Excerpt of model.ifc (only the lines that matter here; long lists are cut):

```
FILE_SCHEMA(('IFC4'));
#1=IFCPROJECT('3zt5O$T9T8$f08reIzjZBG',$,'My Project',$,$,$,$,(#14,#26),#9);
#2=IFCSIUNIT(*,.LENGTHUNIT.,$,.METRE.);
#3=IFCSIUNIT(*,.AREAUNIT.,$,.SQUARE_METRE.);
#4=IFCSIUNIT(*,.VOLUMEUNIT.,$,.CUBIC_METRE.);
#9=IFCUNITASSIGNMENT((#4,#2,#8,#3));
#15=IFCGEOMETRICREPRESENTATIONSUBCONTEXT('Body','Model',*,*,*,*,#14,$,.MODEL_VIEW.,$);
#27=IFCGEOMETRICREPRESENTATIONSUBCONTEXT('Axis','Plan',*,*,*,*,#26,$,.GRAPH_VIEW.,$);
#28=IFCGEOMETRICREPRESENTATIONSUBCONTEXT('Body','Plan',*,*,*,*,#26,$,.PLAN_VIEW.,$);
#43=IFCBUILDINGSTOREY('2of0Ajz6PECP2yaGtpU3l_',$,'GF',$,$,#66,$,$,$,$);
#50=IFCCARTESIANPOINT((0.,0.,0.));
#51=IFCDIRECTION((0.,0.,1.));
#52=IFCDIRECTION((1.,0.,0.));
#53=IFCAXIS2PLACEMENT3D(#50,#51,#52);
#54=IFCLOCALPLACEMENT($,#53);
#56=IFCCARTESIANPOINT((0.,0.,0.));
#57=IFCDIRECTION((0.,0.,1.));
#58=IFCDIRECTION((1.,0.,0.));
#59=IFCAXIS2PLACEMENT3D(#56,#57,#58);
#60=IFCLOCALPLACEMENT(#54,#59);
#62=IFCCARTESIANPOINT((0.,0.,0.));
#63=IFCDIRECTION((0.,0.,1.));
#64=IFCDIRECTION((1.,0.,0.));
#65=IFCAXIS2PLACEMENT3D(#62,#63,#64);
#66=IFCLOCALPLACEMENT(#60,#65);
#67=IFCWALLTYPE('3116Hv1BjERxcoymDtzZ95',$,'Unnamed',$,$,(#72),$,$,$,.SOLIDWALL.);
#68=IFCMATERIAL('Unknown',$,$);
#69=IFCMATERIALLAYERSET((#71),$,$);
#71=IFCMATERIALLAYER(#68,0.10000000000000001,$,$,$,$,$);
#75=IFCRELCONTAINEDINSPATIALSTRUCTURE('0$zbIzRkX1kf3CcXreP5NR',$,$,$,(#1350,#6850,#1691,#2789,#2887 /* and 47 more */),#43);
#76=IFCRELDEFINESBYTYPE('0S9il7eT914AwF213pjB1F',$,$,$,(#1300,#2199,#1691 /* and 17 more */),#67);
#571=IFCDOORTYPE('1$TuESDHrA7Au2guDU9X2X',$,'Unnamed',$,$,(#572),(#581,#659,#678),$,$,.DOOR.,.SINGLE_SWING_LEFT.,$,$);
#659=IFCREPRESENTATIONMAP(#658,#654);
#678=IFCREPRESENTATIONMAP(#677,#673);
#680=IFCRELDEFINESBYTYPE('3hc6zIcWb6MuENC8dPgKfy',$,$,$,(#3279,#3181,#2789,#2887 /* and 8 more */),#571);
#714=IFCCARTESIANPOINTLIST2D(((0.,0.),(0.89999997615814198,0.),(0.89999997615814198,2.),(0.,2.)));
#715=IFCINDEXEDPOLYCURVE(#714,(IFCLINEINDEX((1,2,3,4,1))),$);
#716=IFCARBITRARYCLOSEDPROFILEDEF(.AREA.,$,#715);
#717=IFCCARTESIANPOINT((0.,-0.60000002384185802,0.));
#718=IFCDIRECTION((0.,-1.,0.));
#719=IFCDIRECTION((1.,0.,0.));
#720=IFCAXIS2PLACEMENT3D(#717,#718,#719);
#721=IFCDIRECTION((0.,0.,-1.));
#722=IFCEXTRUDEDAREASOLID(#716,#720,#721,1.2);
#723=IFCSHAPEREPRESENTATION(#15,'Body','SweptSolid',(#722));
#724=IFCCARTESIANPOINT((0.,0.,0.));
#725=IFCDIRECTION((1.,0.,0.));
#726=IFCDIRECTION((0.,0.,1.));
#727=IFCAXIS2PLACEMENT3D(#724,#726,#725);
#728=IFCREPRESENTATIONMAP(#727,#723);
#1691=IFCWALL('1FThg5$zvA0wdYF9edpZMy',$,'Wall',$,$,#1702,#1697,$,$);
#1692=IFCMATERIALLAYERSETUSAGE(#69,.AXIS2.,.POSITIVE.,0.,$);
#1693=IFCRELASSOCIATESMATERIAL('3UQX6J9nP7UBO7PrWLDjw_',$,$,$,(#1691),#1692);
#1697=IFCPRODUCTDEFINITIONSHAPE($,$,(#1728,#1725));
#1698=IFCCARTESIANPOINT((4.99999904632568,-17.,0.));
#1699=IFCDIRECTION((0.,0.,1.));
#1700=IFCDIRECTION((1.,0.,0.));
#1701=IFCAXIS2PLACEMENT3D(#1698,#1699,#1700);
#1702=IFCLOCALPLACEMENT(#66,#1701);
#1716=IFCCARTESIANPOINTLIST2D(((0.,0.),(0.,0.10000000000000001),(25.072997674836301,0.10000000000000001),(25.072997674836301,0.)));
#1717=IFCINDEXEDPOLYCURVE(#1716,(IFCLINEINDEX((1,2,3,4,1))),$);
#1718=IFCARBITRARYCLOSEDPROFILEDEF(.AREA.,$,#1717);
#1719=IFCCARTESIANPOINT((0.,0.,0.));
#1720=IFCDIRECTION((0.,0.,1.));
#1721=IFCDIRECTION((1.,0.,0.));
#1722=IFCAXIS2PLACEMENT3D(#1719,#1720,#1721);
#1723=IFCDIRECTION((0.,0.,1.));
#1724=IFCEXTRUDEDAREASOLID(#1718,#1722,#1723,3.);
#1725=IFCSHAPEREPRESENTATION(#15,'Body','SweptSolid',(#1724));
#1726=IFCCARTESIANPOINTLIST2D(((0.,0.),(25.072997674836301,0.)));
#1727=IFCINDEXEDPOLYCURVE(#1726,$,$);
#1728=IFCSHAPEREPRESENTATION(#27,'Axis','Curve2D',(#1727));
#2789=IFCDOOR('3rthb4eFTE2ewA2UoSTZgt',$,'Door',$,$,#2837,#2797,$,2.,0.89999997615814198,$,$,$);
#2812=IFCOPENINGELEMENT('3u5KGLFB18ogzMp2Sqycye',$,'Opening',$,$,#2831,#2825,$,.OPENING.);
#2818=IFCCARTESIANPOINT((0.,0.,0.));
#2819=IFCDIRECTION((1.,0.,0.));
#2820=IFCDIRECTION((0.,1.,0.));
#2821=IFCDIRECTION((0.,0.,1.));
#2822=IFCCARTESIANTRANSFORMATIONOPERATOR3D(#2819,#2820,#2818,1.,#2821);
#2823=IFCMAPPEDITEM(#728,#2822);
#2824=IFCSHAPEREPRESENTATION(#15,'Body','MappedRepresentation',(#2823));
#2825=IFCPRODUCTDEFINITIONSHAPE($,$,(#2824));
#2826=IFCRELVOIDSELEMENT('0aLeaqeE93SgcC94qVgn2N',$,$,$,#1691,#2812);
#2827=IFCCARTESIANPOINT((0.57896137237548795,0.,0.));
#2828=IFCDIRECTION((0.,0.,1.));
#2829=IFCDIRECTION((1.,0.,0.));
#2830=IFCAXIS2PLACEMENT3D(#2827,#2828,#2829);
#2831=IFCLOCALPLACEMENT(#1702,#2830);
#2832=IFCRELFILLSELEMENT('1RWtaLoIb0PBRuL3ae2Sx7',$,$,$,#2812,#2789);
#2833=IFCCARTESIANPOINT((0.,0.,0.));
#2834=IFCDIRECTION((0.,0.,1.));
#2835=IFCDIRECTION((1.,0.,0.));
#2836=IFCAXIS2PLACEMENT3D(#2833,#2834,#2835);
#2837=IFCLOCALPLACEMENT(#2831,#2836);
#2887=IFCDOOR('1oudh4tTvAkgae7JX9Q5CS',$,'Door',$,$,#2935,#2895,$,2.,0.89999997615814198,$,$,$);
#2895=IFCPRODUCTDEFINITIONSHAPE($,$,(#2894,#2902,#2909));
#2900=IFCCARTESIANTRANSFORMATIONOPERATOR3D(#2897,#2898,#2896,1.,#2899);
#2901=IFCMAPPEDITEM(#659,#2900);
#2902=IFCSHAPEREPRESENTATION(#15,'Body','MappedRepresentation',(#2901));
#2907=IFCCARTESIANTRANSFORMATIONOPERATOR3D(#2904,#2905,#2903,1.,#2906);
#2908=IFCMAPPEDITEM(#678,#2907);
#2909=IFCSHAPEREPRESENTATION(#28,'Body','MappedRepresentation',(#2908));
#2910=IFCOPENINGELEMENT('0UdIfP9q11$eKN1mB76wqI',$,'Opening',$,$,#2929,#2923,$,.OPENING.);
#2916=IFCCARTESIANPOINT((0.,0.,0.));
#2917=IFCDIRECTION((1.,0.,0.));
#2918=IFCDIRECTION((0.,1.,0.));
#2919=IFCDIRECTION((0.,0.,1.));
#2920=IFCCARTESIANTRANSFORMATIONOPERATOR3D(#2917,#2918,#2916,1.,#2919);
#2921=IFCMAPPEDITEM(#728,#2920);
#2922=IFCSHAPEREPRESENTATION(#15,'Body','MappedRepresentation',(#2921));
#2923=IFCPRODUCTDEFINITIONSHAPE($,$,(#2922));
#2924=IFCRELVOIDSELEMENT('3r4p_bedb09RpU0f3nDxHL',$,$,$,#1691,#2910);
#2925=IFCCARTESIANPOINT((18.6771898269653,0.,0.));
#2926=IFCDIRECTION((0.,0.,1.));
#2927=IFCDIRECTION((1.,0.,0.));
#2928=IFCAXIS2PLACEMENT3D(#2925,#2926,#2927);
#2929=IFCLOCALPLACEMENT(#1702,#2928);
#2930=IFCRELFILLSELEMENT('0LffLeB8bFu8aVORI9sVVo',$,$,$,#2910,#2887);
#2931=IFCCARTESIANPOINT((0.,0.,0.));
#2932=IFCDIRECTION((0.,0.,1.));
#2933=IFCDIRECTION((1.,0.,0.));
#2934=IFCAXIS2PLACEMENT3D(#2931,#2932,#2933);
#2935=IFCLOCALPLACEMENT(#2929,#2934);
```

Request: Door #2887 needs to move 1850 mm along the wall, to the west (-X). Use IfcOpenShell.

```python
import ifcopenshell
import ifcopenshell.api.geometry
import ifcopenshell.util.placement

model = ifcopenshell.open("model.ifc")

door = model.by_guid("1oudh4tTvAkgae7JX9Q5CS")
opening = door.FillsVoids[0].RelatingOpeningElement
wall = opening.VoidsElements[0].RelatingBuildingElement

wall_matrix = ifcopenshell.util.placement.get_local_placement(wall.ObjectPlacement)
shift = wall_matrix[:3, 0] * -1.85
before = ifcopenshell.util.placement.get_local_placement(door.ObjectPlacement)[:3, 3].copy()

# The door is placed relative to its opening, so it follows when the opening moves.
matrix = ifcopenshell.util.placement.get_local_placement(opening.ObjectPlacement)
matrix[:3, 3] += shift
ifcopenshell.api.geometry.edit_object_placement(
    model, product=opening, matrix=matrix, is_si=False, should_transform_children=True
)

after = ifcopenshell.util.placement.get_local_placement(door.ObjectPlacement)[:3, 3]
print("door moved by", (after - before).round(3) + 0.0)

model.write("model_updated.ifc")
```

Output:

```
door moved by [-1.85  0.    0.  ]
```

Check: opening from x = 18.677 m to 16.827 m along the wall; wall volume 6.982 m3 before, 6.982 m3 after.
